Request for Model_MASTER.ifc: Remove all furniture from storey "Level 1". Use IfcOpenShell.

First a look at what the model holds.

```python
import ifcopenshell
import ifcopenshell.util.element

model = ifcopenshell.open("Model_MASTER.ifc")
print(model.schema)
storey = next(s for s in model.by_type("IfcBuildingStorey") if s.Name == "Level 1")
furniture = [e for e in ifcopenshell.util.element.get_decomposition(storey) if e.is_a("IfcFurnishingElement")]
seen = {}
for e in furniture:
    element_type = ifcopenshell.util.element.get_type(e)
    name = element_type.Name if element_type not in (None, e) else None
    seen[name] = seen.get(name, 0) + 1
for name, count in sorted(seen.items(), key=str):
    print(count, "x", name)
```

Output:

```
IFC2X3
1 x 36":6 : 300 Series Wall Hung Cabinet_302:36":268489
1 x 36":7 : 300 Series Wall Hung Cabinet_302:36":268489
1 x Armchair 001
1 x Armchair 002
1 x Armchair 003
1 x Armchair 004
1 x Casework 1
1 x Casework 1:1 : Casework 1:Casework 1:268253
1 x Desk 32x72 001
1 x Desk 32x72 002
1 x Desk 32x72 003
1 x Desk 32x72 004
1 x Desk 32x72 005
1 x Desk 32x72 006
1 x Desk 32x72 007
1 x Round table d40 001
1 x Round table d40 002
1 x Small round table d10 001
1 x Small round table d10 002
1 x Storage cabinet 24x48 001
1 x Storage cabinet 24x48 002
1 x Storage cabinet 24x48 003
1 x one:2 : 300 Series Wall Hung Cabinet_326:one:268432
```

```python
import ifcopenshell
import ifcopenshell.api.root
import ifcopenshell.util.element

model = ifcopenshell.open("Model_MASTER.ifc")

storey = next(s for s in model.by_type("IfcBuildingStorey") if s.Name == "Level 1")
furniture = [e for e in ifcopenshell.util.element.get_decomposition(storey) if e.is_a("IfcFurnishingElement")]

for e in furniture:
    ifcopenshell.api.root.remove_product(model, product=e)
print(len(furniture), "removed")

model.write("Model_MASTER_rev.ifc")
```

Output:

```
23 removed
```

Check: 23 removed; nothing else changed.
